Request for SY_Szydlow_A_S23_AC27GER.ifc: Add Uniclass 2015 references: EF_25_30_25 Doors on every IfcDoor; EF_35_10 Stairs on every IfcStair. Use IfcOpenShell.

First a look at what the model holds.

```python
import ifcopenshell

model = ifcopenshell.open("SY_Szydlow_A_S23_AC27GER.ifc")
print(model.schema)
print("classifications:", [c.Name for c in model.by_type("IfcClassification")])
for ifc_class in ("IfcDoor", "IfcRoof", "IfcStair", "IfcWall", "IfcWindow"):
    print(ifc_class, len(model.by_type(ifc_class)))
```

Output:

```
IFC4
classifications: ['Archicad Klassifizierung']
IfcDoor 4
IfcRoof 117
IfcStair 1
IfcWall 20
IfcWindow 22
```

```python
import ifcopenshell
import ifcopenshell.api.classification

model = ifcopenshell.open("SY_Szydlow_A_S23_AC27GER.ifc")

system = ifcopenshell.api.classification.add_classification(model, classification="Uniclass 2015")

codes = {
    "IfcDoor": ("EF_25_30_25", "Doors"),
    "IfcStair": ("EF_35_10", "Stairs"),
}
for ifc_class, (code, name) in codes.items():
    products = model.by_type(ifc_class)
    ifcopenshell.api.classification.add_reference(
        model, products=products, classification=system, identification=code, name=name
    )
    print(code, len(products))

model.write("SY_Szydlow_A_S23_AC27GER-out.ifc")
```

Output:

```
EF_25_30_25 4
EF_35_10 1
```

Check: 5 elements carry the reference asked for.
